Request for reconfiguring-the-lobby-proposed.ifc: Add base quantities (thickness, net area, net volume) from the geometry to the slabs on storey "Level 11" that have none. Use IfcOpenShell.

First a look at what the model holds.

```python
import ifcopenshell
import ifcopenshell.util.element
import ifcopenshell.util.unit

model = ifcopenshell.open("reconfiguring-the-lobby-proposed.ifc")
print(model.schema)
for unit_type in ("LENGTHUNIT", "AREAUNIT", "VOLUMEUNIT"):
    print(unit_type, ifcopenshell.util.unit.calculate_unit_scale(model, unit_type))
storey = next(s for s in model.by_type("IfcBuildingStorey") if s.Name == "Level 11")
slabs = [e for e in ifcopenshell.util.element.get_decomposition(storey) if e.is_a("IfcSlab")]
for e in sorted(slabs, key=lambda e: e.id()):
    print(e.id(), e.is_a(), e.Name, list(ifcopenshell.util.element.get_psets(e, qtos_only=True)), sep=" | ")
```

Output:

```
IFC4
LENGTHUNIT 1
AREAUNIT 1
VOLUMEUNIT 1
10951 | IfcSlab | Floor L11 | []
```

```python
import ifcopenshell
import ifcopenshell.api.pset
import ifcopenshell.geom
import ifcopenshell.util.element
import ifcopenshell.util.shape
import ifcopenshell.util.unit

model = ifcopenshell.open("reconfiguring-the-lobby-proposed.ifc")
unit_scale = ifcopenshell.util.unit.calculate_unit_scale(model)
area_scale = ifcopenshell.util.unit.calculate_unit_scale(model, "AREAUNIT")
volume_scale = ifcopenshell.util.unit.calculate_unit_scale(model, "VOLUMEUNIT")
settings = ifcopenshell.geom.settings()

storey = next(s for s in model.by_type("IfcBuildingStorey") if s.Name == "Level 11")
slabs = [e for e in ifcopenshell.util.element.get_decomposition(storey) if e.is_a("IfcSlab")]

for e in sorted(slabs, key=lambda e: e.id()):
    if ifcopenshell.util.element.get_psets(e, qtos_only=True, should_inherit=False):
        continue
    # Geometry comes back in metres, in the element's own axes.
    shape = ifcopenshell.geom.create_shape(settings, e)
    values = {
        "Width": ifcopenshell.util.shape.get_z(shape.geometry) / unit_scale,
        "NetArea": ifcopenshell.util.shape.get_footprint_area(shape.geometry) / area_scale,
        "NetVolume": ifcopenshell.util.shape.get_volume(shape.geometry) / volume_scale,
    }
    qto = ifcopenshell.api.pset.add_qto(model, product=e, name="Qto_SlabBaseQuantities")
    ifcopenshell.api.pset.edit_qto(model, qto=qto, properties=values)
    print(e.id(), {k: round(v, 3) for k, v in values.items()})

model.write("reconfiguring-the-lobby-proposed-out.ifc")
```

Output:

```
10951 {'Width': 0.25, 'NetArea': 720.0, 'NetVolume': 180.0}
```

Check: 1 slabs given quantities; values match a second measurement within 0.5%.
